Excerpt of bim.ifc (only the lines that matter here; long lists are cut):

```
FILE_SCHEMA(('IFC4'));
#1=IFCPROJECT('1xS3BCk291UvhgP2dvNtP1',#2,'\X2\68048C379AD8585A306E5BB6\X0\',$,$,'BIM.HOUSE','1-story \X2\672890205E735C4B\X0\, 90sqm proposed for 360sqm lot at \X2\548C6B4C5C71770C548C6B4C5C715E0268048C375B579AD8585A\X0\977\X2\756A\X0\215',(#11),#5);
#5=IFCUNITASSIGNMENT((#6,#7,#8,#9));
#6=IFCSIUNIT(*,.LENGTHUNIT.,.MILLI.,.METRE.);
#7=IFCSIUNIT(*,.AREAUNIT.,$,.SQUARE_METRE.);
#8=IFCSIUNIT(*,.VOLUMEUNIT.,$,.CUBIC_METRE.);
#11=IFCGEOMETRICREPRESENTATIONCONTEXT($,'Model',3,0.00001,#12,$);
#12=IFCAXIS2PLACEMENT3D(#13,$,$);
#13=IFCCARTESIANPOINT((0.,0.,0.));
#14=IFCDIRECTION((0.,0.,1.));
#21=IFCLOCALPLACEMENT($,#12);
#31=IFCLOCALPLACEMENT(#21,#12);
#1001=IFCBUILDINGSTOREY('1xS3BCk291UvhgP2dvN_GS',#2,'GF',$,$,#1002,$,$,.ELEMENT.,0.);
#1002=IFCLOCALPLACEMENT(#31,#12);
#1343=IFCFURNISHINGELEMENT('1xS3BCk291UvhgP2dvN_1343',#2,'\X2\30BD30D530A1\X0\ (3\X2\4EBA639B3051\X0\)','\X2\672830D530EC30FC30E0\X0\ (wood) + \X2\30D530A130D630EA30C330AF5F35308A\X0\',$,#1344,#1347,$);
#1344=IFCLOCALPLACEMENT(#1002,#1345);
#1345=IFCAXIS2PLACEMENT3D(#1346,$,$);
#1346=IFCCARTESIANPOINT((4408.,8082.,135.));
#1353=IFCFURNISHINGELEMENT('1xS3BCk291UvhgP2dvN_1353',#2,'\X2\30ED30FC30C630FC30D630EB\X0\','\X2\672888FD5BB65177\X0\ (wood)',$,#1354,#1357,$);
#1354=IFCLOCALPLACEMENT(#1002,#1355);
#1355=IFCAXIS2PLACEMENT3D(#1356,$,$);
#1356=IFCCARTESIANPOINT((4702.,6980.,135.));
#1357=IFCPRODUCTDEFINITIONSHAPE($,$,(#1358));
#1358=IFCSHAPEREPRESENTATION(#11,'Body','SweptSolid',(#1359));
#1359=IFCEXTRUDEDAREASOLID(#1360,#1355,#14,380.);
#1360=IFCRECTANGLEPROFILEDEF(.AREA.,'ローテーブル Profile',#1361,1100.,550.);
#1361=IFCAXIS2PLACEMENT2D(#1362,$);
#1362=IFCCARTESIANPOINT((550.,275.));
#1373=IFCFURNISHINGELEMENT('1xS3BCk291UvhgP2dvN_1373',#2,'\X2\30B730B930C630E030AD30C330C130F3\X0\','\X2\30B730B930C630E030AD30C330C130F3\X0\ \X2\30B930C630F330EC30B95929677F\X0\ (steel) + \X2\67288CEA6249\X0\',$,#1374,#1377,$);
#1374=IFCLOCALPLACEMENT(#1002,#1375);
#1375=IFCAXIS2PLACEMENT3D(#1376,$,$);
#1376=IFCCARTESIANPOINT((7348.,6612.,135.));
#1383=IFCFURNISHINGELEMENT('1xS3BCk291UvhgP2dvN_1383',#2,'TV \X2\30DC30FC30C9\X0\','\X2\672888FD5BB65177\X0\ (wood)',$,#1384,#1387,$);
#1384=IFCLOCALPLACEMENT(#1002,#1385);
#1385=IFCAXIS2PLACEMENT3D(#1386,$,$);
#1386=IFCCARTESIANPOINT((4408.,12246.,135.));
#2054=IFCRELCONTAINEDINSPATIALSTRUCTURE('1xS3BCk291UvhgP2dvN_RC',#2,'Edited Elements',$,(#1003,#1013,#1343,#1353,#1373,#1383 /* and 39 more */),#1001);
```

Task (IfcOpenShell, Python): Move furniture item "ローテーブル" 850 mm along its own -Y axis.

```python
import ifcopenshell
import ifcopenshell.api.geometry
import ifcopenshell.util.placement

model = ifcopenshell.open("bim.ifc")

item = model.by_guid("1xS3BCk291UvhgP2dvN_1353")
matrix = ifcopenshell.util.placement.get_local_placement(item.ObjectPlacement)
matrix[:3, 3] -= matrix[:3, 1] * 850.0
ifcopenshell.api.geometry.edit_object_placement(model, product=item, matrix=matrix, is_si=False)

print(ifcopenshell.util.placement.get_local_placement(item.ObjectPlacement).round(3) + 0.0)

model.write("bim-out.ifc")
```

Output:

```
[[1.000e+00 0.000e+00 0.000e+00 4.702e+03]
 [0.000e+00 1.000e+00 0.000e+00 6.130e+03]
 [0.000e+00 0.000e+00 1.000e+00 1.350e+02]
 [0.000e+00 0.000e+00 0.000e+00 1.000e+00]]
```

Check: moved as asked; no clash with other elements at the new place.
